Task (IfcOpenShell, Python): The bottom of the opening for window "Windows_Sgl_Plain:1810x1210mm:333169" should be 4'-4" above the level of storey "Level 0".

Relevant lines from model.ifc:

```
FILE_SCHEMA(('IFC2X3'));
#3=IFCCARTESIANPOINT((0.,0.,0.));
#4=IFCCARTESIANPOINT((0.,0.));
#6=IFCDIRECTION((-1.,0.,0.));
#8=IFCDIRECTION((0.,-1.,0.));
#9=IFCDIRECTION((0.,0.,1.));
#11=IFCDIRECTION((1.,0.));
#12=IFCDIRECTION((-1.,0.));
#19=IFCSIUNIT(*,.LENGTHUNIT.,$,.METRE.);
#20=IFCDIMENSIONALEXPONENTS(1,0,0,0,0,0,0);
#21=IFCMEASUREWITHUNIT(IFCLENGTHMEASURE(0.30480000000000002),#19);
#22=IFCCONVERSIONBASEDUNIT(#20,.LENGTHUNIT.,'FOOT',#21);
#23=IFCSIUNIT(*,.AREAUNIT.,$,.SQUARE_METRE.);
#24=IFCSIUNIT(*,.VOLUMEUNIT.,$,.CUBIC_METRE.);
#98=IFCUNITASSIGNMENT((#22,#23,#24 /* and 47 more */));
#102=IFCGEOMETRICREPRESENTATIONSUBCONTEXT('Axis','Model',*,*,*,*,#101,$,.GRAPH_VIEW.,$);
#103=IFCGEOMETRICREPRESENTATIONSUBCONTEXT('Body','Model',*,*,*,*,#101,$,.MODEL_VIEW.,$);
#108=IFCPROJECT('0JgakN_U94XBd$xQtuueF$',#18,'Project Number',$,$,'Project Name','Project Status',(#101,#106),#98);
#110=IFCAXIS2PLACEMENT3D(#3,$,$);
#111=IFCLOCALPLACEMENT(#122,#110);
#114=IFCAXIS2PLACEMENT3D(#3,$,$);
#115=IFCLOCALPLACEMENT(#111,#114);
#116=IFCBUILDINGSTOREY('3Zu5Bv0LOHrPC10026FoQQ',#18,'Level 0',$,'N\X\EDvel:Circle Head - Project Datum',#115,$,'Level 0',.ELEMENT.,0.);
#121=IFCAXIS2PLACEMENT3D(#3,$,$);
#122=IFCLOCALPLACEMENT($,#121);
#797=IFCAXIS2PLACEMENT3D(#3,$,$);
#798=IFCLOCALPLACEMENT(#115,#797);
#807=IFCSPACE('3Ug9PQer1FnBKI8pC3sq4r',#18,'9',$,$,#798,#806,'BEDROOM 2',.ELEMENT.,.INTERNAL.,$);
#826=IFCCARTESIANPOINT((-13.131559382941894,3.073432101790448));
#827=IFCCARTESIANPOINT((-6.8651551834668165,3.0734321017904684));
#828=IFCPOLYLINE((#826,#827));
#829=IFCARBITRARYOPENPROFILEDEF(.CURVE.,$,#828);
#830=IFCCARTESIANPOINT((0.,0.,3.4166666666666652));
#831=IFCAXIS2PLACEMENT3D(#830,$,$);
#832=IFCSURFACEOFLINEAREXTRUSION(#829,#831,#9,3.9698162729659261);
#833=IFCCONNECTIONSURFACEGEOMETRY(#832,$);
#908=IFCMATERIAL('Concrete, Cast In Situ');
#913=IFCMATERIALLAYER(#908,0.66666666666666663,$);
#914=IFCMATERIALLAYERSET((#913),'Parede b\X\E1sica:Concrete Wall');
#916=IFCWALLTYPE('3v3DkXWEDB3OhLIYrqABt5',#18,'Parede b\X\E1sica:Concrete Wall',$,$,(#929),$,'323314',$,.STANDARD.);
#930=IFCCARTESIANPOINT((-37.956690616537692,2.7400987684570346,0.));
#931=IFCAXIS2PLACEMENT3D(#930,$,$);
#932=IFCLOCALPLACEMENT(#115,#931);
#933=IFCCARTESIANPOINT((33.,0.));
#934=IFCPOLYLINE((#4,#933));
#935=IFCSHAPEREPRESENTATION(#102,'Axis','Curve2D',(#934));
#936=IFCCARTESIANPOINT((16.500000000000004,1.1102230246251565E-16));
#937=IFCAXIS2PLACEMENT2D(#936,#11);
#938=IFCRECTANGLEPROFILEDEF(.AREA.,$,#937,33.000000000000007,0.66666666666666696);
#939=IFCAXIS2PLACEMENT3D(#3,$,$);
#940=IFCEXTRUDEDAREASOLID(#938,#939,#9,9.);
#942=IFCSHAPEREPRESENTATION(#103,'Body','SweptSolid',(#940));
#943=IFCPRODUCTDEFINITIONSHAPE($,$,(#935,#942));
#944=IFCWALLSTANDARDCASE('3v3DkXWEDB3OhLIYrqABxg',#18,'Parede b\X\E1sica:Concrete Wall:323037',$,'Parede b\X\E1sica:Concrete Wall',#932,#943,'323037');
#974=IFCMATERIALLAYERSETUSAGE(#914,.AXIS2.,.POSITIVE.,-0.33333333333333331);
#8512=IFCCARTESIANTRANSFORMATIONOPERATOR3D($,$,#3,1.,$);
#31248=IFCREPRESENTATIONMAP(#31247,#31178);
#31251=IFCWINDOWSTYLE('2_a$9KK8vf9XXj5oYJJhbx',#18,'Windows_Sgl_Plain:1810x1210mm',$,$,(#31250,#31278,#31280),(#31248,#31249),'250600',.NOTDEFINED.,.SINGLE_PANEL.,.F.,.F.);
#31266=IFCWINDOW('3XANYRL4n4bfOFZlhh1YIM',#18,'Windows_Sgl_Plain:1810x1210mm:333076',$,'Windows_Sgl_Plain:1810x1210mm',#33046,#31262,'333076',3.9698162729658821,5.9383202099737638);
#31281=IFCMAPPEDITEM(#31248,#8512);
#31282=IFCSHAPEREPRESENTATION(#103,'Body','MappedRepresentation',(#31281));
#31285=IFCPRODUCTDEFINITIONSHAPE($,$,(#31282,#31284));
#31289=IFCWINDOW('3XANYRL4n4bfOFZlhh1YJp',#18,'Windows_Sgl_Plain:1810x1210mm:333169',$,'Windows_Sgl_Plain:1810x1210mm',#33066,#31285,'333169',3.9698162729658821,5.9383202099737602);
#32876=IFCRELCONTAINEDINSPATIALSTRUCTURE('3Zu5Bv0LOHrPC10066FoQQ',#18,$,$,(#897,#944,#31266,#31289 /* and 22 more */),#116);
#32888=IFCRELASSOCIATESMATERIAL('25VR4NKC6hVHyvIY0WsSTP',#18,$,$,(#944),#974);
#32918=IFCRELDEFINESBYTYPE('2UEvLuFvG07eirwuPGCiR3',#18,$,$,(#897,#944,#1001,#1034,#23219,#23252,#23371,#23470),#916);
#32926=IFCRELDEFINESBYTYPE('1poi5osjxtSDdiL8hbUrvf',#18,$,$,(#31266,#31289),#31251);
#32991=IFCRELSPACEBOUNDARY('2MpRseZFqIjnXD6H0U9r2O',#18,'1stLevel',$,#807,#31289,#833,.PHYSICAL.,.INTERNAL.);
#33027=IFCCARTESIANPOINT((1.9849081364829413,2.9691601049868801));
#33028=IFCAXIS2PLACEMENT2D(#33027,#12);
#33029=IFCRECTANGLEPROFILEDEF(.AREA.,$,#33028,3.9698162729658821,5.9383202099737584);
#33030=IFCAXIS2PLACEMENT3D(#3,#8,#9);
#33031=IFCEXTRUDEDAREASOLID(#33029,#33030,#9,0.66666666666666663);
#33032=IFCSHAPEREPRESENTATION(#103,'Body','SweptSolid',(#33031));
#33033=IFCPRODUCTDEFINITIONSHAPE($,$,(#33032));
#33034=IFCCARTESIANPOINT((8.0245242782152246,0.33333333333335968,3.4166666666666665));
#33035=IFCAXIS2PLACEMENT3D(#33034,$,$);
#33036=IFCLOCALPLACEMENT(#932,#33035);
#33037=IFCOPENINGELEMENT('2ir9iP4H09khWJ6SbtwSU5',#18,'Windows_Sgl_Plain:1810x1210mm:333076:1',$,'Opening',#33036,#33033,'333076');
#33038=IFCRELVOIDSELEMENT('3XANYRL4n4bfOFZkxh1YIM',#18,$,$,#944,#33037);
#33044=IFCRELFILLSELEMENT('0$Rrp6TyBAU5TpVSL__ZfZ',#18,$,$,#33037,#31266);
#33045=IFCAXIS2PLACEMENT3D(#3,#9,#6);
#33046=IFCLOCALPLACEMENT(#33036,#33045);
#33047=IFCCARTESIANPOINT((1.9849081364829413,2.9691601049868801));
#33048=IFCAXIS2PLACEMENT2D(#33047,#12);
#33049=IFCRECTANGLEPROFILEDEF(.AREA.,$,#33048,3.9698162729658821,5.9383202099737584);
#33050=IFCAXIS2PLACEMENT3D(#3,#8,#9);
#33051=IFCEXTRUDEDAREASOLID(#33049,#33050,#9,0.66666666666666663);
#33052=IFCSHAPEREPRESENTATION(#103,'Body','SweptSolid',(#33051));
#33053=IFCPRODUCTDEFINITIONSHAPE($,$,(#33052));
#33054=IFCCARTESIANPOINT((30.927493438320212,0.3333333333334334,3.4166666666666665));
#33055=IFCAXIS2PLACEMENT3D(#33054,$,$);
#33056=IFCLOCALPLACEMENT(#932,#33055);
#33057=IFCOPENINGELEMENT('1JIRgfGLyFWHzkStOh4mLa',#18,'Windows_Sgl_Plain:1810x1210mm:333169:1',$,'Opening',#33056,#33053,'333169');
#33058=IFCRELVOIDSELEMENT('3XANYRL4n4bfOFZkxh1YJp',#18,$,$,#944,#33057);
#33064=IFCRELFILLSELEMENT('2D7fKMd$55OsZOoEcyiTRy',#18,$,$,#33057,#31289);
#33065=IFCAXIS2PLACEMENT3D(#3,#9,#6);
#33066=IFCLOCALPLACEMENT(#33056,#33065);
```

```python
import numpy as np
import ifcopenshell
import ifcopenshell.api.geometry
import ifcopenshell.geom
import ifcopenshell.util.element
import ifcopenshell.util.placement
import ifcopenshell.util.shape
import ifcopenshell.util.unit

model = ifcopenshell.open("model.ifc")
unit_scale = ifcopenshell.util.unit.calculate_unit_scale(model)

window = model.by_guid("3XANYRL4n4bfOFZlhh1YJp")
opening = window.FillsVoids[0].RelatingOpeningElement
storey = ifcopenshell.util.element.get_container(window, ifc_class="IfcBuildingStorey")
level = ifcopenshell.util.placement.get_local_placement(storey.ObjectPlacement)[2, 3]

# The opening's origin need not be at the sill, so measure its lowest point.
shape = ifcopenshell.geom.create_shape(ifcopenshell.geom.settings(), opening)
bottom = ifcopenshell.util.shape.get_shape_bottom_elevation(shape, shape.geometry) / unit_scale
dz = level + 52 * 0.0254 / unit_scale - bottom

shift = np.array([0.0, 0.0, dz])
# The window is placed relative to its opening, so it follows when the opening moves.
matrix = ifcopenshell.util.placement.get_local_placement(opening.ObjectPlacement)
matrix[:3, 3] += shift
ifcopenshell.api.geometry.edit_object_placement(
    model, product=opening, matrix=matrix, is_si=False, should_transform_children=True
)

# Space boundary surfaces are stored in each space's coordinates; move them too.
for rel in window.ProvidesBoundaries:
    if not rel.ConnectionGeometry:
        continue
    surface = rel.ConnectionGeometry.SurfaceOnRelatingElement
    space_matrix = ifcopenshell.util.placement.get_local_placement(rel.RelatingSpace.ObjectPlacement)
    point = np.array(surface.Position.Location.Coordinates) + space_matrix[:3, :3].T @ shift
    surface.Position = model.createIfcAxis2Placement3D(
        model.createIfcCartesianPoint(point.tolist()), surface.Position.Axis, surface.Position.RefDirection
    )

print(f"moved by {dz * unit_scale:+.3f} m")

model.write("model_rev.ifc")
```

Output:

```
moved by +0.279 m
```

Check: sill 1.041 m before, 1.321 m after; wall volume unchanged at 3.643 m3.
